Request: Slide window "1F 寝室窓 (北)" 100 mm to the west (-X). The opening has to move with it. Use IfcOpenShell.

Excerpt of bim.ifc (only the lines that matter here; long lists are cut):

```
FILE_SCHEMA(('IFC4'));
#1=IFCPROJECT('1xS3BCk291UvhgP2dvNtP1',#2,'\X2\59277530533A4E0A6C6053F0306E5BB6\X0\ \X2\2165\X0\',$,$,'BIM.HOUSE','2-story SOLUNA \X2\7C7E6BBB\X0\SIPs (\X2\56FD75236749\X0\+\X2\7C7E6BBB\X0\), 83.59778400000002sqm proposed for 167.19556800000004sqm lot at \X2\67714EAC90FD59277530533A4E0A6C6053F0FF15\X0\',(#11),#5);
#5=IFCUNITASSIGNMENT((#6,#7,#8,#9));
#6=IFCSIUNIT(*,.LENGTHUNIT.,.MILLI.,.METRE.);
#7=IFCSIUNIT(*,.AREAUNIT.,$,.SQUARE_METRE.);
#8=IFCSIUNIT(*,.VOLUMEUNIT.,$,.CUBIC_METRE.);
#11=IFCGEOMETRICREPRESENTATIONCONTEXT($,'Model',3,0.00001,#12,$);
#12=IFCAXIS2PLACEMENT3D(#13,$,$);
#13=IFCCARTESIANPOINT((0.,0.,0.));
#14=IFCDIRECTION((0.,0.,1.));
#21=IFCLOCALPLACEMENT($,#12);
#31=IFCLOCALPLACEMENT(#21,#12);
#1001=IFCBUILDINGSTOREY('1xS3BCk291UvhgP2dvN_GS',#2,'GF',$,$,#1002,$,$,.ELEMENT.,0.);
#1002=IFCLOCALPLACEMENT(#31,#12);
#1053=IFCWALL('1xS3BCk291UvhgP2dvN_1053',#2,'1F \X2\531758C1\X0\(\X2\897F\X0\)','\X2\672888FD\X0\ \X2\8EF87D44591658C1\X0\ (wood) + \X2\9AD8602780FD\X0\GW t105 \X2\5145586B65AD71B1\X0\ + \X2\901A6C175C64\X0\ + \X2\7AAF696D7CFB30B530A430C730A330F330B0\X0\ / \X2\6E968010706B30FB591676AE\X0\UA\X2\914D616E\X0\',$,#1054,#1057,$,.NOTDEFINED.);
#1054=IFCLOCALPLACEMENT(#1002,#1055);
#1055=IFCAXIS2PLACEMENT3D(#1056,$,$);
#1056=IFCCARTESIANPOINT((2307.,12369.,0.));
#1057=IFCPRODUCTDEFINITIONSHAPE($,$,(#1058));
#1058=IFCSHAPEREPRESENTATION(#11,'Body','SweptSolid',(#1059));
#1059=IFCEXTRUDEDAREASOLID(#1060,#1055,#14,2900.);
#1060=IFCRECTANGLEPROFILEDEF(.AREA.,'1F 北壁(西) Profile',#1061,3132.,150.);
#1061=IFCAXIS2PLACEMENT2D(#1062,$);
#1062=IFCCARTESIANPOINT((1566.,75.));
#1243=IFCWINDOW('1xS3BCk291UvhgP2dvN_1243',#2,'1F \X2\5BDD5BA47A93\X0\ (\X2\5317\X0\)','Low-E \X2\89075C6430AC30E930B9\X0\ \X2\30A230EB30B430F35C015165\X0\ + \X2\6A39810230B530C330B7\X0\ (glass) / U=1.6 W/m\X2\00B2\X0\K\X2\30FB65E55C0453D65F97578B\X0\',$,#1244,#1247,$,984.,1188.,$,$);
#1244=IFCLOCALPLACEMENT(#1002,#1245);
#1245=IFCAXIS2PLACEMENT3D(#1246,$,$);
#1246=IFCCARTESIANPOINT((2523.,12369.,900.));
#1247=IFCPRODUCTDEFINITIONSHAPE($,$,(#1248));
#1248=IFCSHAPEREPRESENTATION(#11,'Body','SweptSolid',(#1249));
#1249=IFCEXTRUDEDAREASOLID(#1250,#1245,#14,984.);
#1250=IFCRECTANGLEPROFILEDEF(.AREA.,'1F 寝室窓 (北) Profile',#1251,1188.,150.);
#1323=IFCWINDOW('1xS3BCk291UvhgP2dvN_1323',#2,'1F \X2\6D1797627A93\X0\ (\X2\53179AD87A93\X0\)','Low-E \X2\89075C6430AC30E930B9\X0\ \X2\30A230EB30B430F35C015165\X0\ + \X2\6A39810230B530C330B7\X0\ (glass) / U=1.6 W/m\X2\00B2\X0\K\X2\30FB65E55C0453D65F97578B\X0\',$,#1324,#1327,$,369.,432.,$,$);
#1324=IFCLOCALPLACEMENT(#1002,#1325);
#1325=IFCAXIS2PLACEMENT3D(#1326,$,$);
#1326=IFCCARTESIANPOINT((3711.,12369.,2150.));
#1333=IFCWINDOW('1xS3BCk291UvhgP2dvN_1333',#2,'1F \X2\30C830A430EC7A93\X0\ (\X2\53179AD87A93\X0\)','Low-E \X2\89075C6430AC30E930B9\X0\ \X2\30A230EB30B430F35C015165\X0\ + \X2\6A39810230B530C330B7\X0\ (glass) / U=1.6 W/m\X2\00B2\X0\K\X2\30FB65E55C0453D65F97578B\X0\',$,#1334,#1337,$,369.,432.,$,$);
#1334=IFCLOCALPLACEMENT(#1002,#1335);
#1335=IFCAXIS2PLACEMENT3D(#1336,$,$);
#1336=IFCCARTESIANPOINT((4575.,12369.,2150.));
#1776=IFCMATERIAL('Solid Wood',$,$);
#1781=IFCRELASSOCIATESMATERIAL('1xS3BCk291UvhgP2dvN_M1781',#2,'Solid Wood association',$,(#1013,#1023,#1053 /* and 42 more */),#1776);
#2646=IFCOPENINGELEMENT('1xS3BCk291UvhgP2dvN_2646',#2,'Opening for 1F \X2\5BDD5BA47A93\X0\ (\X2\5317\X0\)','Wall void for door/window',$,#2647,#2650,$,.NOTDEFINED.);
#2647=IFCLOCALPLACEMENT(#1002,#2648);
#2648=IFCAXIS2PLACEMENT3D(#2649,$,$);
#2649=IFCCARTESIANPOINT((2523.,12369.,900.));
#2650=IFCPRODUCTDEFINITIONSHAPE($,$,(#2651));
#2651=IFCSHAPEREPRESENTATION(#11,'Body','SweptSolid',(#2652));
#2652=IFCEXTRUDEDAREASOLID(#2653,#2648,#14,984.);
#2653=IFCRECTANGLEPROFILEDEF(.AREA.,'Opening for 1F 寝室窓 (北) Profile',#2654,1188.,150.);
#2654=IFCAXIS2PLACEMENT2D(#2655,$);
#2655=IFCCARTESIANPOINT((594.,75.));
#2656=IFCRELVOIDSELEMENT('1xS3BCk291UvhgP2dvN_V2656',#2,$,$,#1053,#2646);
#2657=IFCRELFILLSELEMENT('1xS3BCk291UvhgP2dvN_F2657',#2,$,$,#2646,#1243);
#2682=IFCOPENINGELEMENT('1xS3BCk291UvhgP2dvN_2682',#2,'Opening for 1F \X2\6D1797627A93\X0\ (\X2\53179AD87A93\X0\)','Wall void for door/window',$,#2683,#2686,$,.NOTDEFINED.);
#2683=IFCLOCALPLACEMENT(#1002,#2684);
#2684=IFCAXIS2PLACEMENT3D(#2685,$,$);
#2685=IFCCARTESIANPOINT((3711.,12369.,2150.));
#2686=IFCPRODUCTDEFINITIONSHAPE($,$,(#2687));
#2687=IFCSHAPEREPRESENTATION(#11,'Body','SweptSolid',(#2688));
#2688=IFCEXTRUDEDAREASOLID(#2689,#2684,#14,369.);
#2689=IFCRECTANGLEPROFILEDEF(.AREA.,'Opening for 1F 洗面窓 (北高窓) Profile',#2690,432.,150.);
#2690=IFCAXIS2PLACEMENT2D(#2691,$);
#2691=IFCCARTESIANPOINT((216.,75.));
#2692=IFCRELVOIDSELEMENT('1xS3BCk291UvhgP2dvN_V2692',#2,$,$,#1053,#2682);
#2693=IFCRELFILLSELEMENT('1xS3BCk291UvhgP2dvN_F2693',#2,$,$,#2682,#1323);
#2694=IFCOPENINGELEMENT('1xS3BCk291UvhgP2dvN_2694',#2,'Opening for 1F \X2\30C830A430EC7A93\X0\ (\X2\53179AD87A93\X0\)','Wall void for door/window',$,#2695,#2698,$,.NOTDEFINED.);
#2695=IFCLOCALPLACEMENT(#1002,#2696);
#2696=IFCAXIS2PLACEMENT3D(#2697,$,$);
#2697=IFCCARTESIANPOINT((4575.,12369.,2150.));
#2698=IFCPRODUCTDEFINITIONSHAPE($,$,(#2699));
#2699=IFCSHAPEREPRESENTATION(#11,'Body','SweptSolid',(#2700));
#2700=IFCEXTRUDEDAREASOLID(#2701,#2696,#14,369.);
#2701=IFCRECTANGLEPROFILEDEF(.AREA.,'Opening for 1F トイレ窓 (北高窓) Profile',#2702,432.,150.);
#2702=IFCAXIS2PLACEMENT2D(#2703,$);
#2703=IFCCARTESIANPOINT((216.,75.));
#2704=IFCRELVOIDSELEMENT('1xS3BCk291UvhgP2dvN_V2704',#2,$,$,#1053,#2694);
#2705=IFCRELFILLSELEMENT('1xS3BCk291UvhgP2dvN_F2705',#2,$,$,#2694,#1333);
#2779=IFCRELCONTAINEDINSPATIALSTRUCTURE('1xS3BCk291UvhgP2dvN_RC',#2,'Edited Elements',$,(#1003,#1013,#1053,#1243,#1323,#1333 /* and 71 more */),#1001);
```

```python
import ifcopenshell
import ifcopenshell.api.geometry
import ifcopenshell.util.placement
import ifcopenshell.util.unit

model = ifcopenshell.open("bim.ifc")
unit_scale = ifcopenshell.util.unit.calculate_unit_scale(model)

window = model.by_id(1243)
opening = window.FillsVoids[0].RelatingOpeningElement
wall = opening.VoidsElements[0].RelatingBuildingElement

wall_matrix = ifcopenshell.util.placement.get_local_placement(wall.ObjectPlacement)
shift = wall_matrix[:3, 0] * -0.1 / unit_scale
before = ifcopenshell.util.placement.get_local_placement(window.ObjectPlacement)[:3, 3].copy()

# The window is not placed relative to its opening, so move both.
for product in (opening, window):
    matrix = ifcopenshell.util.placement.get_local_placement(product.ObjectPlacement)
    matrix[:3, 3] += shift
    ifcopenshell.api.geometry.edit_object_placement(model, product=product, matrix=matrix, is_si=False)

after = ifcopenshell.util.placement.get_local_placement(window.ObjectPlacement)[:3, 3]
print("window moved by", (after - before).round(3) + 0.0)

model.write("bim_updated.ifc")
```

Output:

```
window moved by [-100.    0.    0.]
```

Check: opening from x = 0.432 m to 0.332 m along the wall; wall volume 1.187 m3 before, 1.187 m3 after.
